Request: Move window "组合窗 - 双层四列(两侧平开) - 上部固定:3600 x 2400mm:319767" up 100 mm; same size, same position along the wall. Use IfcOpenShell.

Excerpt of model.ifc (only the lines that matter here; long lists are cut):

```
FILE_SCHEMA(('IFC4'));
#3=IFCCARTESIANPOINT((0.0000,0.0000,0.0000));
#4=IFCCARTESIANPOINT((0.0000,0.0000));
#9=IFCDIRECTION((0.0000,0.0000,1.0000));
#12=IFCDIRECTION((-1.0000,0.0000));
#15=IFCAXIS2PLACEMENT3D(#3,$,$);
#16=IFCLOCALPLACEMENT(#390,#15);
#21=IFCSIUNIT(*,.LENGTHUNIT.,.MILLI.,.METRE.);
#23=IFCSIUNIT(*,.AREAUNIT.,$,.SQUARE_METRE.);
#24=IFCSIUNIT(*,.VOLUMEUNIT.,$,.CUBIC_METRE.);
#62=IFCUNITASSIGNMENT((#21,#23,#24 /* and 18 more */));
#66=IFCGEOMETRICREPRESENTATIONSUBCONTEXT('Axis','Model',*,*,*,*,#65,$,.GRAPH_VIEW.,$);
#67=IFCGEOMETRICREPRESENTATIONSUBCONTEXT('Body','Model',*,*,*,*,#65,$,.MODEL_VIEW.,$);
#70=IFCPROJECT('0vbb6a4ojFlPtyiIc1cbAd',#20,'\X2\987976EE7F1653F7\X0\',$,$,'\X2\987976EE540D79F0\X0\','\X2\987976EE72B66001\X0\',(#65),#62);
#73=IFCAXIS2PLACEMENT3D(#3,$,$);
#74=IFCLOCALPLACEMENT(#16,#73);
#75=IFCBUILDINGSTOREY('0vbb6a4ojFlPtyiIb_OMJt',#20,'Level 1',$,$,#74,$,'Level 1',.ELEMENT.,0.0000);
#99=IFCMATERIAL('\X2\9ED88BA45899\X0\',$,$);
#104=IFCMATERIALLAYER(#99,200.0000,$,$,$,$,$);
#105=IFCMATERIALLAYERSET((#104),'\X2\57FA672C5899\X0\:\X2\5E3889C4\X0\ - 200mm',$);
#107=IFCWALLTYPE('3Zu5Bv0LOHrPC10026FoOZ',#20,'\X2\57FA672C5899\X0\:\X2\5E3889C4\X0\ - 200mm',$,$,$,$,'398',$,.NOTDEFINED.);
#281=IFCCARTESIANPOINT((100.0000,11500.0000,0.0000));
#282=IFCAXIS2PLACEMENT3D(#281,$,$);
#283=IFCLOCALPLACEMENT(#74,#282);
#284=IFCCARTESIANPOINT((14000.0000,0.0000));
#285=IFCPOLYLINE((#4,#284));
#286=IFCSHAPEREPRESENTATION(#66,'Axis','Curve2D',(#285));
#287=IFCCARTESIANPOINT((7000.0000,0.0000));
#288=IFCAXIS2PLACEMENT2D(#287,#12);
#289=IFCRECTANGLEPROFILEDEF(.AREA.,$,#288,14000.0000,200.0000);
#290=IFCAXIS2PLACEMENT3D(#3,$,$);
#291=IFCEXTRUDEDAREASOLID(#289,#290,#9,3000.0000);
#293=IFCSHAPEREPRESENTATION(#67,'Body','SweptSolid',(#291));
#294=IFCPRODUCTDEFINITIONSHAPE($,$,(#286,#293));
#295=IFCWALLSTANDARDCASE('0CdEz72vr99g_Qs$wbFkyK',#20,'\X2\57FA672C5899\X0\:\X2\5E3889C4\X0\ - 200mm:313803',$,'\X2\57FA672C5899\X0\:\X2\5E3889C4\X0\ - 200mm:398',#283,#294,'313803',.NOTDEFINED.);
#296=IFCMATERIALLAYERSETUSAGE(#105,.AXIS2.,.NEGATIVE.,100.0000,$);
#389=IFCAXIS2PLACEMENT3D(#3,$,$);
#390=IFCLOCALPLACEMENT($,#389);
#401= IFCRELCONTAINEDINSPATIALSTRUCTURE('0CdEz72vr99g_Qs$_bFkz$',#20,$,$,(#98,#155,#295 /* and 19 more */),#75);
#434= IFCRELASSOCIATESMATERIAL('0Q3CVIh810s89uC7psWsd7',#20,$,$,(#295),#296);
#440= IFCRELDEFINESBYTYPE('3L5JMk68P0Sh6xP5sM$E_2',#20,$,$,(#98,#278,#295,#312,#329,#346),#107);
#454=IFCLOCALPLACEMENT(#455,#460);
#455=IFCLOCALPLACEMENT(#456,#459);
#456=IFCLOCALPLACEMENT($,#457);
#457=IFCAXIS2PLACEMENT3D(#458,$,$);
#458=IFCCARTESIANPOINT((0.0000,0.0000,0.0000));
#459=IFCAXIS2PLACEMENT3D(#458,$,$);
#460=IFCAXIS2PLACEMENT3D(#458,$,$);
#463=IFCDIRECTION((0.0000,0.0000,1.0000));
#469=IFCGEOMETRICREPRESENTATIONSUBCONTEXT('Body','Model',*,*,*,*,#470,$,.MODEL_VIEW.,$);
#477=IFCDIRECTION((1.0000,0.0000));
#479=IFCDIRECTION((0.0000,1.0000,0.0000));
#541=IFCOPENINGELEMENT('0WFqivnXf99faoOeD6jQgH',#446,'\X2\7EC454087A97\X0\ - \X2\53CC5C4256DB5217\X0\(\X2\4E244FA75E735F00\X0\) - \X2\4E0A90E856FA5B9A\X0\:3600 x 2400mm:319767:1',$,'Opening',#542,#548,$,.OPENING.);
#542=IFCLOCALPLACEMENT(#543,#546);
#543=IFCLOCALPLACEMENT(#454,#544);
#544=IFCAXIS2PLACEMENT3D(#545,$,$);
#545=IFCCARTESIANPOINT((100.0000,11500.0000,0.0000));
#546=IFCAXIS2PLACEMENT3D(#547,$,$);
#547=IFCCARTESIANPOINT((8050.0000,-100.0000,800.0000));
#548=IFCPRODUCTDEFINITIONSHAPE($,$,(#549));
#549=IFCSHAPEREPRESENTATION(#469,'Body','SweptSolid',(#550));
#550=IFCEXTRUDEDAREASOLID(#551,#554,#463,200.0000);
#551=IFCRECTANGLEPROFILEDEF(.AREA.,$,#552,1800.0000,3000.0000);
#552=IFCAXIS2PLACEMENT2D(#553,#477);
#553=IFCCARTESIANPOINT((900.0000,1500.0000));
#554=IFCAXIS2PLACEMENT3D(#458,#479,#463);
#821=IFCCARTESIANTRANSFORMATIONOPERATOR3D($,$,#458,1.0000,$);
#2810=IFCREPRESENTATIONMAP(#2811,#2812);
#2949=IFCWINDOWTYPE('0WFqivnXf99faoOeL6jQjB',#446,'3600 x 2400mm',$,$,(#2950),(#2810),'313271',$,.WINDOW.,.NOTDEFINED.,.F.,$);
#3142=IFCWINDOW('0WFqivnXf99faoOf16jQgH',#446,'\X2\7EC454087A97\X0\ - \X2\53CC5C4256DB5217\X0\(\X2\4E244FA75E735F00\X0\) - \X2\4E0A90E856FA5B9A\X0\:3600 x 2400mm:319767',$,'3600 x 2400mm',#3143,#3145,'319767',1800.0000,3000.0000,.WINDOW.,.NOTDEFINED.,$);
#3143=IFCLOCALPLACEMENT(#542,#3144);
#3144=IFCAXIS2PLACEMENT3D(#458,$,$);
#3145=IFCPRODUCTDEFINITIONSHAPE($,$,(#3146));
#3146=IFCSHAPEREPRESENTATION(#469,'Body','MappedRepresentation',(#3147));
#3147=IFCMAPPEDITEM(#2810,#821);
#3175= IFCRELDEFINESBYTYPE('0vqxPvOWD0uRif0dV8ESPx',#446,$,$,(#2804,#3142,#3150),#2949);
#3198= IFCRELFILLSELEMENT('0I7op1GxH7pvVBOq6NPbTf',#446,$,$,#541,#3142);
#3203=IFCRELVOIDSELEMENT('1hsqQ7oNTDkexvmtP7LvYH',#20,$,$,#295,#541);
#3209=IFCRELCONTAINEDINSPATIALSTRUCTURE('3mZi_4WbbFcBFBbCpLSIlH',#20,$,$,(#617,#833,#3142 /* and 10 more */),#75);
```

```python
import numpy as np
import ifcopenshell
import ifcopenshell.api.geometry
import ifcopenshell.util.placement
import ifcopenshell.util.unit

model = ifcopenshell.open("model.ifc")
unit_scale = ifcopenshell.util.unit.calculate_unit_scale(model)

window = model.by_guid("0WFqivnXf99faoOf16jQgH")
opening = window.FillsVoids[0].RelatingOpeningElement
dz = 0.1 / unit_scale

shift = np.array([0.0, 0.0, dz])
# The window is placed relative to its opening, so it follows when the opening moves.
matrix = ifcopenshell.util.placement.get_local_placement(opening.ObjectPlacement)
matrix[:3, 3] += shift
ifcopenshell.api.geometry.edit_object_placement(
    model, product=opening, matrix=matrix, is_si=False, should_transform_children=True
)

print(f"moved by {dz * unit_scale:+.3f} m")

model.write("model_edited.ifc")
```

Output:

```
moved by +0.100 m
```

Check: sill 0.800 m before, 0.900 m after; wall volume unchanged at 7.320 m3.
